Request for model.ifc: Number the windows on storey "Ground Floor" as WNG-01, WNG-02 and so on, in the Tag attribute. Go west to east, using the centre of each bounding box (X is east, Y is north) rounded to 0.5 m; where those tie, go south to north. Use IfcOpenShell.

First a look at what the model holds.

```python
import ifcopenshell
import ifcopenshell.util.element
import ifcopenshell.util.placement

model = ifcopenshell.open("model.ifc")
print(model.schema)
storey = next(s for s in model.by_type("IfcBuildingStorey") if s.Name == "Ground Floor")
windows = [e for e in ifcopenshell.util.element.get_decomposition(storey) if e.is_a("IfcWindow")]
for e in sorted(windows, key=lambda e: e.id()):
    origin = ifcopenshell.util.placement.get_local_placement(e.ObjectPlacement)[:3, 3]
    print(e.id(), e.Tag, e.Name, origin.round(2) + 0.0, sep=" | ")
```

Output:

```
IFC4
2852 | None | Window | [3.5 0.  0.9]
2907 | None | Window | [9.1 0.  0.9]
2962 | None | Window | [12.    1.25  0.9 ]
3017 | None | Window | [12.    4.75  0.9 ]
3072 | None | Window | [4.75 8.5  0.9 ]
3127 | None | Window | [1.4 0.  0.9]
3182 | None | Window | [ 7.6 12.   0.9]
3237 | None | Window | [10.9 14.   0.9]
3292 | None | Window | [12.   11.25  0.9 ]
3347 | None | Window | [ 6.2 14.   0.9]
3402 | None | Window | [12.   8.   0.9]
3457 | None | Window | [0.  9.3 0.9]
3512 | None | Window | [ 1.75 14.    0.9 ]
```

```python
import ifcopenshell
import ifcopenshell.geom
import ifcopenshell.util.element
import ifcopenshell.util.shape

model = ifcopenshell.open("model.ifc")
settings = ifcopenshell.geom.settings()
settings.set("use-world-coords", True)


def centre(element):
    shape = ifcopenshell.geom.create_shape(settings, element)
    return ifcopenshell.util.shape.get_bbox_centroid(shape.geometry)


storey = next(s for s in model.by_type("IfcBuildingStorey") if s.Name == "Ground Floor")
windows = [e for e in ifcopenshell.util.element.get_decomposition(storey) if e.is_a("IfcWindow")]

# Insertion points can sit at a corner or the storey origin, so sort by the geometry (in metres).
centres = {e: centre(e) for e in windows}
windows.sort(key=lambda e: (round(centres[e][0] / 0.5), centres[e][1]))

for i, e in enumerate(windows, start=1):
    number = f"WNG-{i:02d}"
    e.Tag = number
    print(e.id(), number)

model.write("model_updated.ifc")
```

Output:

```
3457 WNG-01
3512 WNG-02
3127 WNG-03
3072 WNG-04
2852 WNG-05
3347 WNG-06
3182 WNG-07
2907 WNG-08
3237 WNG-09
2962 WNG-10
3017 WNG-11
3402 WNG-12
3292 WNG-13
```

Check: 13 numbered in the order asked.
